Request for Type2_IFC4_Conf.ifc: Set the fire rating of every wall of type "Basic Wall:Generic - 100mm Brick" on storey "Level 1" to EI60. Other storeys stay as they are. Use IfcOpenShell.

First a look at what the model holds.

```python
import ifcopenshell
import ifcopenshell.util.element

model = ifcopenshell.open("Type2_IFC4_Conf.ifc")
print(model.schema)
storey = next(s for s in model.by_type("IfcBuildingStorey") if s.Name == "Level 1")
walls = [e for e in ifcopenshell.util.element.get_decomposition(storey) if e.is_a("IfcWall")]
seen = {}
for e in walls:
    element_type = ifcopenshell.util.element.get_type(e)
    key = (element_type.Name if element_type != e and element_type else None, ifcopenshell.util.element.get_pset(e, "Pset_WallCommon", "FireRating"))
    seen[key] = seen.get(key, 0) + 1
for (name, value), count in sorted(seen.items(), key=str):
    print(count, "x", name, "|", value)
```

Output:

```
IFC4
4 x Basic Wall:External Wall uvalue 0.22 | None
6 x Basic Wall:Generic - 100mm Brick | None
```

```python
import ifcopenshell
import ifcopenshell.api.pset
import ifcopenshell.util.element

model = ifcopenshell.open("Type2_IFC4_Conf.ifc")

storey = next(s for s in model.by_type("IfcBuildingStorey") if s.Name == "Level 1")
walls = [e for e in ifcopenshell.util.element.get_decomposition(storey) if e.is_a("IfcWall")]

count = 0
for e in walls:
    element_type = ifcopenshell.util.element.get_type(e)
    if element_type in (None, e) or element_type.Name != "Basic Wall:Generic - 100mm Brick":
        continue
    # add_pset returns the element's existing set when there is one.
    pset = ifcopenshell.api.pset.add_pset(model, product=e, name="Pset_WallCommon")
    ifcopenshell.api.pset.edit_pset(model, pset=pset, properties={"FireRating": "EI60"})
    count += 1

print(count, "walls updated")

model.write("Type2_IFC4_Conf_v2.ifc")
```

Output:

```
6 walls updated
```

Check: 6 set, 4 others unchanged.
